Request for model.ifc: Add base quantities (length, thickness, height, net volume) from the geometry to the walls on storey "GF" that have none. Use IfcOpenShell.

First a look at what the model holds.

```python
import ifcopenshell
import ifcopenshell.util.element
import ifcopenshell.util.unit

model = ifcopenshell.open("model.ifc")
print(model.schema)
for unit_type in ("LENGTHUNIT", "AREAUNIT", "VOLUMEUNIT"):
    print(unit_type, ifcopenshell.util.unit.calculate_unit_scale(model, unit_type))
storey = next(s for s in model.by_type("IfcBuildingStorey") if s.Name == "GF")
walls = [e for e in ifcopenshell.util.element.get_decomposition(storey) if e.is_a("IfcWall")]
for e in sorted(walls, key=lambda e: e.id()):
    print(e.id(), e.is_a(), e.Name, list(ifcopenshell.util.element.get_psets(e, qtos_only=True)), sep=" | ")
```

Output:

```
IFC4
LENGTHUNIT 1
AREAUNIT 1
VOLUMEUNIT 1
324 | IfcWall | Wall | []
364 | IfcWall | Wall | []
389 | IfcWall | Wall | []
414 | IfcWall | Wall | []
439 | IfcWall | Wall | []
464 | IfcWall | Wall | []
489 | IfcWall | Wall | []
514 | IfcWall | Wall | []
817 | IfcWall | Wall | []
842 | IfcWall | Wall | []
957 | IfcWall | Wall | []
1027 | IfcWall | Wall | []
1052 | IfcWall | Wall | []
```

```python
import ifcopenshell
import ifcopenshell.api.pset
import ifcopenshell.geom
import ifcopenshell.util.element
import ifcopenshell.util.shape
import ifcopenshell.util.unit

model = ifcopenshell.open("model.ifc")
unit_scale = ifcopenshell.util.unit.calculate_unit_scale(model)
volume_scale = ifcopenshell.util.unit.calculate_unit_scale(model, "VOLUMEUNIT")
settings = ifcopenshell.geom.settings()

storey = next(s for s in model.by_type("IfcBuildingStorey") if s.Name == "GF")
walls = [e for e in ifcopenshell.util.element.get_decomposition(storey) if e.is_a("IfcWall")]

for e in sorted(walls, key=lambda e: e.id()):
    if ifcopenshell.util.element.get_psets(e, qtos_only=True, should_inherit=False):
        continue
    # Geometry comes back in metres, in the element's own axes.
    shape = ifcopenshell.geom.create_shape(settings, e)
    values = {
        "Length": ifcopenshell.util.shape.get_x(shape.geometry) / unit_scale,
        "Width": ifcopenshell.util.shape.get_y(shape.geometry) / unit_scale,
        "Height": ifcopenshell.util.shape.get_z(shape.geometry) / unit_scale,
        "NetVolume": ifcopenshell.util.shape.get_volume(shape.geometry) / volume_scale,
    }
    qto = ifcopenshell.api.pset.add_qto(model, product=e, name="Qto_WallBaseQuantities")
    ifcopenshell.api.pset.edit_qto(model, qto=qto, properties=values)
    print(e.id(), {k: round(v, 3) for k, v in values.items()})

model.write("model_edited.ifc")
```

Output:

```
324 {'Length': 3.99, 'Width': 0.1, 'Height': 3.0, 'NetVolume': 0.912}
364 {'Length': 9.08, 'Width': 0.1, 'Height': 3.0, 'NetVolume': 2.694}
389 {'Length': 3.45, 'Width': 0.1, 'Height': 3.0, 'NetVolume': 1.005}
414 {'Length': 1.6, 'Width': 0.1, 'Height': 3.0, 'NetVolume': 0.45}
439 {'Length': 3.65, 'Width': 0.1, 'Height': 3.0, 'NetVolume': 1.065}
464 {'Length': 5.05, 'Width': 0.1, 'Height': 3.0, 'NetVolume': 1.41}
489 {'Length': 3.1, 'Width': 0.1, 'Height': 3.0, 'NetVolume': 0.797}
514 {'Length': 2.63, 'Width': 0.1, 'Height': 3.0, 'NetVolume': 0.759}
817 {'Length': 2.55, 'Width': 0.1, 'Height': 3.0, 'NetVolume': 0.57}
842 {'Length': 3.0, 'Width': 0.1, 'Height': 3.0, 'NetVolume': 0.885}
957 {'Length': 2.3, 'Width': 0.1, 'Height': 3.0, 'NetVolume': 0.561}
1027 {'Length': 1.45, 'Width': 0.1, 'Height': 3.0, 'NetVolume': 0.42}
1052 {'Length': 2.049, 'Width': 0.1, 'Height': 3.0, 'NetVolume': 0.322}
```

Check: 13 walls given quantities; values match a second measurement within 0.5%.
